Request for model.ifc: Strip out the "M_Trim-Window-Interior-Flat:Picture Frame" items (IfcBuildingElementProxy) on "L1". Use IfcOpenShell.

First a look at what the model holds.

```python
import ifcopenshell
import ifcopenshell.util.element

model = ifcopenshell.open("model.ifc")
print(model.schema)
storey = next(s for s in model.by_type("IfcBuildingStorey") if s.Name == "L1")
proxies = [e for e in ifcopenshell.util.element.get_decomposition(storey) if e.is_a("IfcBuildingElementProxy")]
seen = {}
for e in proxies:
    element_type = ifcopenshell.util.element.get_type(e)
    name = element_type.Name if element_type not in (None, e) else None
    seen[name] = seen.get(name, 0) + 1
for name, count in sorted(seen.items(), key=str):
    print(count, "x", name)
```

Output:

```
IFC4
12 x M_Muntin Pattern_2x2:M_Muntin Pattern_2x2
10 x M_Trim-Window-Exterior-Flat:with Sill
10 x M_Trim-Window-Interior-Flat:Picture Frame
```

```python
import ifcopenshell
import ifcopenshell.api.root
import ifcopenshell.util.element

model = ifcopenshell.open("model.ifc")

storey = next(s for s in model.by_type("IfcBuildingStorey") if s.Name == "L1")
proxies = [e for e in ifcopenshell.util.element.get_decomposition(storey) if e.is_a("IfcBuildingElementProxy")]
targets = [e for e in proxies if (t := ifcopenshell.util.element.get_type(e)) not in (None, e) and t.Name == "M_Trim-Window-Interior-Flat:Picture Frame"]

for e in targets:
    ifcopenshell.api.root.remove_product(model, product=e)
print(len(targets), "removed")

model.write("model_v2.ifc")
```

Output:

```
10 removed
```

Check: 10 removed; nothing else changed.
